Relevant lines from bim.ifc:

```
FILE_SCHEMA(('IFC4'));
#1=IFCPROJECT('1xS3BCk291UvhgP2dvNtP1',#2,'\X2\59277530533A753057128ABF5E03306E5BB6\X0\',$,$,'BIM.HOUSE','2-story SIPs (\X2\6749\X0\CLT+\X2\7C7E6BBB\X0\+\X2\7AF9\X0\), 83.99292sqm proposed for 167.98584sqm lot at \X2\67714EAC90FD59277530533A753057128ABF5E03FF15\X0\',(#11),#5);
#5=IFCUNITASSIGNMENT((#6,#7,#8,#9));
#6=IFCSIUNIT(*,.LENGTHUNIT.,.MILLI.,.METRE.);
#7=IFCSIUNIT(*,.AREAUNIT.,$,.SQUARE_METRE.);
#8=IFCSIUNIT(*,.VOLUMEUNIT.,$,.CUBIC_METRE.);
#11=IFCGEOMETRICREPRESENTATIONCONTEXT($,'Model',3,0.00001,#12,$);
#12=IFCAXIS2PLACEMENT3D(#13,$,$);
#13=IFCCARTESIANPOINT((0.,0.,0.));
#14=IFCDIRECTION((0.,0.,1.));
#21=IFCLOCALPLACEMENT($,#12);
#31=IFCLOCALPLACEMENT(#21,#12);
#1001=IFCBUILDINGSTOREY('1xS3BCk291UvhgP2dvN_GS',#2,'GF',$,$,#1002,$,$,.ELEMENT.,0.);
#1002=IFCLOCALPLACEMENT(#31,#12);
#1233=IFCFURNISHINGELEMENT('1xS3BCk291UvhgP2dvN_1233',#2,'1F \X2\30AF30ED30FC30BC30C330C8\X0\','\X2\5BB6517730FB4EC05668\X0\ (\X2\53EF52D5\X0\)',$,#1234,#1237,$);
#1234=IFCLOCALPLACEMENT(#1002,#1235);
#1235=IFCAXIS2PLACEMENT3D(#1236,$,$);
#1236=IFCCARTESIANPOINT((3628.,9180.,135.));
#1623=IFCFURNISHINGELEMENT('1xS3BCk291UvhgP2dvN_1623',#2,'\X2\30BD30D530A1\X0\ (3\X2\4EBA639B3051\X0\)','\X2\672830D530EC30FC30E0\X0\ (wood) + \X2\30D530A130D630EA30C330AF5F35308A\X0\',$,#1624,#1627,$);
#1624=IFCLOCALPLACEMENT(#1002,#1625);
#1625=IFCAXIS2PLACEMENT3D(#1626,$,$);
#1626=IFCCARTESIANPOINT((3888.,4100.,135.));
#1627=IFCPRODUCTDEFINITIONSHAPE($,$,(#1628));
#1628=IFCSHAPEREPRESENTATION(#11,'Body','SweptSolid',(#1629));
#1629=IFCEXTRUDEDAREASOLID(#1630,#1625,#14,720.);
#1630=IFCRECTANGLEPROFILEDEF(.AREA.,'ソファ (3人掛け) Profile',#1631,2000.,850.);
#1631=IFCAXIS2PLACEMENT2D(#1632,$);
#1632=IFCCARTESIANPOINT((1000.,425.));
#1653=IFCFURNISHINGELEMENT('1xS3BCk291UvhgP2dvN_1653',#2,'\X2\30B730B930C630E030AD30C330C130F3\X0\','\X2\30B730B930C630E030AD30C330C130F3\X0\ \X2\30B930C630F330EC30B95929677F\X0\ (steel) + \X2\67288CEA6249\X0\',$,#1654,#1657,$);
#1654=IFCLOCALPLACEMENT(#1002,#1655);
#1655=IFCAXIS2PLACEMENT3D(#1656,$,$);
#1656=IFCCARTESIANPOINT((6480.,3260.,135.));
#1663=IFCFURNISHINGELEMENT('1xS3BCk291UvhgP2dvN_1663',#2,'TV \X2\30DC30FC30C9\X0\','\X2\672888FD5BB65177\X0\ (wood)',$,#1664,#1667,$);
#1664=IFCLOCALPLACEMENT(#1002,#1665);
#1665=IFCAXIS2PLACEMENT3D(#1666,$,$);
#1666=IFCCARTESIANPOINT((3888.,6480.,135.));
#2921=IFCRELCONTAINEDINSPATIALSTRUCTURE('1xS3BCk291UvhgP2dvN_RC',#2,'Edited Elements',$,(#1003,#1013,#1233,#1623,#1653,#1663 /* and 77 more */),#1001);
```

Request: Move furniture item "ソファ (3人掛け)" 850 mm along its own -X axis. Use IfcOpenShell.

```python
import ifcopenshell
import ifcopenshell.api.geometry
import ifcopenshell.util.placement

model = ifcopenshell.open("bim.ifc")

item = model.by_id(1623)
matrix = ifcopenshell.util.placement.get_local_placement(item.ObjectPlacement)
matrix[:3, 3] -= matrix[:3, 0] * 850.0
ifcopenshell.api.geometry.edit_object_placement(model, product=item, matrix=matrix, is_si=False)

print(ifcopenshell.util.placement.get_local_placement(item.ObjectPlacement).round(3) + 0.0)

model.write("bim-out.ifc")
```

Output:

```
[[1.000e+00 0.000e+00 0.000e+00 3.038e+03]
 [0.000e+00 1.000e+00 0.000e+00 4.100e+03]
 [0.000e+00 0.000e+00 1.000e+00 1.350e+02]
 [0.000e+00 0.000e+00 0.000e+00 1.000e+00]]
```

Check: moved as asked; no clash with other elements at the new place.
